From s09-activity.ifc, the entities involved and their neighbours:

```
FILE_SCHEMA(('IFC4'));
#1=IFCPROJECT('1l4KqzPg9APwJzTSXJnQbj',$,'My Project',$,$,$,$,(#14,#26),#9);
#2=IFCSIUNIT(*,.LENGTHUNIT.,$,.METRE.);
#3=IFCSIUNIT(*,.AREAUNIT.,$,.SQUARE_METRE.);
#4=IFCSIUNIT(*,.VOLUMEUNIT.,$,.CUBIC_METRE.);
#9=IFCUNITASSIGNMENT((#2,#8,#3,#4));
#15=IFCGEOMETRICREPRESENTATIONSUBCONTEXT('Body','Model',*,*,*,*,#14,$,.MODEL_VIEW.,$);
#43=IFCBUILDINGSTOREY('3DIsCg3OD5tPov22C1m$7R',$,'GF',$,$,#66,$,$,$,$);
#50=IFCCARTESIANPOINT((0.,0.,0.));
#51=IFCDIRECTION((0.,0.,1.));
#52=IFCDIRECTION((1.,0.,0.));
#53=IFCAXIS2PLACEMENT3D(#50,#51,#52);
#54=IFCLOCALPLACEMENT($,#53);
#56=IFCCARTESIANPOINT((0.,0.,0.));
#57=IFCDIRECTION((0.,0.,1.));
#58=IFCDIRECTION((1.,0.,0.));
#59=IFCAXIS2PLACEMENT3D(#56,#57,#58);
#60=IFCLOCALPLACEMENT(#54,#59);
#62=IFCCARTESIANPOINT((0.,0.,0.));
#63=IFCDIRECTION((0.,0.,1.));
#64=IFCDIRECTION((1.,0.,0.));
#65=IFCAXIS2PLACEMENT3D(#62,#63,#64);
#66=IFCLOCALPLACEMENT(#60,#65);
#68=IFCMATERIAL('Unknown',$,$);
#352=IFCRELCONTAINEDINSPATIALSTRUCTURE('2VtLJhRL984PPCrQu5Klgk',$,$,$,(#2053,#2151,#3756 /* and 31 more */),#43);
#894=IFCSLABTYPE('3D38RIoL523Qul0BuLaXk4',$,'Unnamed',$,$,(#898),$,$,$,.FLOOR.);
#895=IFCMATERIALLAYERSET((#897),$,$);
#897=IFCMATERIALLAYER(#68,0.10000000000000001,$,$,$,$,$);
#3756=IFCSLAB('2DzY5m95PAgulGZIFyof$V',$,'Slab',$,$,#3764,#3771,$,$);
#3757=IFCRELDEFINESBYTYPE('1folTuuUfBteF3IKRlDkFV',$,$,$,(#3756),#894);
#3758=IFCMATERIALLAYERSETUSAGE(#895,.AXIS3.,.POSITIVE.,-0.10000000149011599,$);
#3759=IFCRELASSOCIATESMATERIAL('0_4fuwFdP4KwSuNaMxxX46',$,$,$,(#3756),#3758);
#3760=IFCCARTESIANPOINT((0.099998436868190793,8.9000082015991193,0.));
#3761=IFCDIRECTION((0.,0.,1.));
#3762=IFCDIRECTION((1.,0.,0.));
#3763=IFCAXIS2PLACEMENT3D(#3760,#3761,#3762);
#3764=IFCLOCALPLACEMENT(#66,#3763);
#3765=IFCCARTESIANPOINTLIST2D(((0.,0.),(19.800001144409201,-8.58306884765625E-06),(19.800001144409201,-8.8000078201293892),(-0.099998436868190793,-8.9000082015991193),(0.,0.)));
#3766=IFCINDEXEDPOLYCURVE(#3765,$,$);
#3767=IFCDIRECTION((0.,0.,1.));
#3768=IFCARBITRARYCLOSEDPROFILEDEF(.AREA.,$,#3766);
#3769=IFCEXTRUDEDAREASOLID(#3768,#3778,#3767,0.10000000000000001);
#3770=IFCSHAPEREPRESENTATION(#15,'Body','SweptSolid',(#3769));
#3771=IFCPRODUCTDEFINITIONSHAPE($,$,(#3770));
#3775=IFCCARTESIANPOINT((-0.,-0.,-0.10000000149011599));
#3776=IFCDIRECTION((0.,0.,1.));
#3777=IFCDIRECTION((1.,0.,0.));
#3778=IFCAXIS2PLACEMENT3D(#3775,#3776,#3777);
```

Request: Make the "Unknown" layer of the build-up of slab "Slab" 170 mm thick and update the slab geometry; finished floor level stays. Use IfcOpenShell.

```python
import ifcopenshell
import ifcopenshell.util.element
import ifcopenshell.util.representation
import ifcopenshell.util.unit

model = ifcopenshell.open("s09-activity.ifc")
unit_scale = ifcopenshell.util.unit.calculate_unit_scale(model)

layer_set = model.by_id(895)
layer = next(l for l in layer_set.MaterialLayers if l.Material and l.Material.Name == "Unknown")
change = 0.17 / unit_scale - layer.LayerThickness
layer.LayerThickness += change

# Geometry does not follow the layer set by itself.
slabs = [e for e in ifcopenshell.util.element.get_elements_by_material(model, layer_set) if e.is_a("IfcSlab")]
for slab in sorted(slabs, key=lambda e: e.id()):
    body = ifcopenshell.util.representation.get_representation(slab, "Model", "Body")
    solid = body.Items[0]
    old_depth = solid.Depth
    solid.Depth += change
    # Extruded upwards: lower the start of the extrusion so the top stays.
    x, y, z = solid.Position.Location.Coordinates
    solid.Position.Location = model.createIfcCartesianPoint((x, y, z - change))
    print(slab.id(), f"{old_depth:g} -> {solid.Depth:g}")

# The layers are counted up from the underside, which has moved.
for usage in {ifcopenshell.util.element.get_material(slab) for slab in slabs}:
    usage.OffsetFromReferenceLine -= change

model.write("s09-activity-out.ifc")
```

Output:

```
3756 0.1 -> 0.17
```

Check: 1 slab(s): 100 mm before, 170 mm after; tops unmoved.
